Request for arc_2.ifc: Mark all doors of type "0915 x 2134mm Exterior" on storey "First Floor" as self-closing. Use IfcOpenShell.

First a look at what the model holds.

```python
import ifcopenshell
import ifcopenshell.util.element

model = ifcopenshell.open("arc_2.ifc")
print(model.schema)
storey = next(s for s in model.by_type("IfcBuildingStorey") if s.Name == "First Floor")
doors = [e for e in ifcopenshell.util.element.get_decomposition(storey) if e.is_a("IfcDoor")]
seen = {}
for e in doors:
    element_type = ifcopenshell.util.element.get_type(e)
    key = (element_type.Name if element_type != e and element_type else None, ifcopenshell.util.element.get_pset(e, "Pset_DoorCommon", "SelfClosing"))
    seen[key] = seen.get(key, 0) + 1
for (name, value), count in sorted(seen.items(), key=str):
    print(count, "x", name, "|", value)
```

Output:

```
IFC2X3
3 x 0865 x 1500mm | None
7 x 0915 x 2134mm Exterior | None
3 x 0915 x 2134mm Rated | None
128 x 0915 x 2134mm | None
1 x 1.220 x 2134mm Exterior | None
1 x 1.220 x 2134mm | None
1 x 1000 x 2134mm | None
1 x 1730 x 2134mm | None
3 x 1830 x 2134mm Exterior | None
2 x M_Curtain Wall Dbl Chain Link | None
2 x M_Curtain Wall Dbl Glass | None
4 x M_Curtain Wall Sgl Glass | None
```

```python
import ifcopenshell
import ifcopenshell.api.pset
import ifcopenshell.util.element

model = ifcopenshell.open("arc_2.ifc")

storey = next(s for s in model.by_type("IfcBuildingStorey") if s.Name == "First Floor")
doors = [e for e in ifcopenshell.util.element.get_decomposition(storey) if e.is_a("IfcDoor")]

count = 0
for e in doors:
    element_type = ifcopenshell.util.element.get_type(e)
    if element_type in (None, e) or element_type.Name != "0915 x 2134mm Exterior":
        continue
    # add_pset returns the element's existing set when there is one.
    pset = ifcopenshell.api.pset.add_pset(model, product=e, name="Pset_DoorCommon")
    ifcopenshell.api.pset.edit_pset(model, pset=pset, properties={"SelfClosing": True})
    count += 1

print(count, "doors updated")

model.write("arc_2_updated.ifc")
```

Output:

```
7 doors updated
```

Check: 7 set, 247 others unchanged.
